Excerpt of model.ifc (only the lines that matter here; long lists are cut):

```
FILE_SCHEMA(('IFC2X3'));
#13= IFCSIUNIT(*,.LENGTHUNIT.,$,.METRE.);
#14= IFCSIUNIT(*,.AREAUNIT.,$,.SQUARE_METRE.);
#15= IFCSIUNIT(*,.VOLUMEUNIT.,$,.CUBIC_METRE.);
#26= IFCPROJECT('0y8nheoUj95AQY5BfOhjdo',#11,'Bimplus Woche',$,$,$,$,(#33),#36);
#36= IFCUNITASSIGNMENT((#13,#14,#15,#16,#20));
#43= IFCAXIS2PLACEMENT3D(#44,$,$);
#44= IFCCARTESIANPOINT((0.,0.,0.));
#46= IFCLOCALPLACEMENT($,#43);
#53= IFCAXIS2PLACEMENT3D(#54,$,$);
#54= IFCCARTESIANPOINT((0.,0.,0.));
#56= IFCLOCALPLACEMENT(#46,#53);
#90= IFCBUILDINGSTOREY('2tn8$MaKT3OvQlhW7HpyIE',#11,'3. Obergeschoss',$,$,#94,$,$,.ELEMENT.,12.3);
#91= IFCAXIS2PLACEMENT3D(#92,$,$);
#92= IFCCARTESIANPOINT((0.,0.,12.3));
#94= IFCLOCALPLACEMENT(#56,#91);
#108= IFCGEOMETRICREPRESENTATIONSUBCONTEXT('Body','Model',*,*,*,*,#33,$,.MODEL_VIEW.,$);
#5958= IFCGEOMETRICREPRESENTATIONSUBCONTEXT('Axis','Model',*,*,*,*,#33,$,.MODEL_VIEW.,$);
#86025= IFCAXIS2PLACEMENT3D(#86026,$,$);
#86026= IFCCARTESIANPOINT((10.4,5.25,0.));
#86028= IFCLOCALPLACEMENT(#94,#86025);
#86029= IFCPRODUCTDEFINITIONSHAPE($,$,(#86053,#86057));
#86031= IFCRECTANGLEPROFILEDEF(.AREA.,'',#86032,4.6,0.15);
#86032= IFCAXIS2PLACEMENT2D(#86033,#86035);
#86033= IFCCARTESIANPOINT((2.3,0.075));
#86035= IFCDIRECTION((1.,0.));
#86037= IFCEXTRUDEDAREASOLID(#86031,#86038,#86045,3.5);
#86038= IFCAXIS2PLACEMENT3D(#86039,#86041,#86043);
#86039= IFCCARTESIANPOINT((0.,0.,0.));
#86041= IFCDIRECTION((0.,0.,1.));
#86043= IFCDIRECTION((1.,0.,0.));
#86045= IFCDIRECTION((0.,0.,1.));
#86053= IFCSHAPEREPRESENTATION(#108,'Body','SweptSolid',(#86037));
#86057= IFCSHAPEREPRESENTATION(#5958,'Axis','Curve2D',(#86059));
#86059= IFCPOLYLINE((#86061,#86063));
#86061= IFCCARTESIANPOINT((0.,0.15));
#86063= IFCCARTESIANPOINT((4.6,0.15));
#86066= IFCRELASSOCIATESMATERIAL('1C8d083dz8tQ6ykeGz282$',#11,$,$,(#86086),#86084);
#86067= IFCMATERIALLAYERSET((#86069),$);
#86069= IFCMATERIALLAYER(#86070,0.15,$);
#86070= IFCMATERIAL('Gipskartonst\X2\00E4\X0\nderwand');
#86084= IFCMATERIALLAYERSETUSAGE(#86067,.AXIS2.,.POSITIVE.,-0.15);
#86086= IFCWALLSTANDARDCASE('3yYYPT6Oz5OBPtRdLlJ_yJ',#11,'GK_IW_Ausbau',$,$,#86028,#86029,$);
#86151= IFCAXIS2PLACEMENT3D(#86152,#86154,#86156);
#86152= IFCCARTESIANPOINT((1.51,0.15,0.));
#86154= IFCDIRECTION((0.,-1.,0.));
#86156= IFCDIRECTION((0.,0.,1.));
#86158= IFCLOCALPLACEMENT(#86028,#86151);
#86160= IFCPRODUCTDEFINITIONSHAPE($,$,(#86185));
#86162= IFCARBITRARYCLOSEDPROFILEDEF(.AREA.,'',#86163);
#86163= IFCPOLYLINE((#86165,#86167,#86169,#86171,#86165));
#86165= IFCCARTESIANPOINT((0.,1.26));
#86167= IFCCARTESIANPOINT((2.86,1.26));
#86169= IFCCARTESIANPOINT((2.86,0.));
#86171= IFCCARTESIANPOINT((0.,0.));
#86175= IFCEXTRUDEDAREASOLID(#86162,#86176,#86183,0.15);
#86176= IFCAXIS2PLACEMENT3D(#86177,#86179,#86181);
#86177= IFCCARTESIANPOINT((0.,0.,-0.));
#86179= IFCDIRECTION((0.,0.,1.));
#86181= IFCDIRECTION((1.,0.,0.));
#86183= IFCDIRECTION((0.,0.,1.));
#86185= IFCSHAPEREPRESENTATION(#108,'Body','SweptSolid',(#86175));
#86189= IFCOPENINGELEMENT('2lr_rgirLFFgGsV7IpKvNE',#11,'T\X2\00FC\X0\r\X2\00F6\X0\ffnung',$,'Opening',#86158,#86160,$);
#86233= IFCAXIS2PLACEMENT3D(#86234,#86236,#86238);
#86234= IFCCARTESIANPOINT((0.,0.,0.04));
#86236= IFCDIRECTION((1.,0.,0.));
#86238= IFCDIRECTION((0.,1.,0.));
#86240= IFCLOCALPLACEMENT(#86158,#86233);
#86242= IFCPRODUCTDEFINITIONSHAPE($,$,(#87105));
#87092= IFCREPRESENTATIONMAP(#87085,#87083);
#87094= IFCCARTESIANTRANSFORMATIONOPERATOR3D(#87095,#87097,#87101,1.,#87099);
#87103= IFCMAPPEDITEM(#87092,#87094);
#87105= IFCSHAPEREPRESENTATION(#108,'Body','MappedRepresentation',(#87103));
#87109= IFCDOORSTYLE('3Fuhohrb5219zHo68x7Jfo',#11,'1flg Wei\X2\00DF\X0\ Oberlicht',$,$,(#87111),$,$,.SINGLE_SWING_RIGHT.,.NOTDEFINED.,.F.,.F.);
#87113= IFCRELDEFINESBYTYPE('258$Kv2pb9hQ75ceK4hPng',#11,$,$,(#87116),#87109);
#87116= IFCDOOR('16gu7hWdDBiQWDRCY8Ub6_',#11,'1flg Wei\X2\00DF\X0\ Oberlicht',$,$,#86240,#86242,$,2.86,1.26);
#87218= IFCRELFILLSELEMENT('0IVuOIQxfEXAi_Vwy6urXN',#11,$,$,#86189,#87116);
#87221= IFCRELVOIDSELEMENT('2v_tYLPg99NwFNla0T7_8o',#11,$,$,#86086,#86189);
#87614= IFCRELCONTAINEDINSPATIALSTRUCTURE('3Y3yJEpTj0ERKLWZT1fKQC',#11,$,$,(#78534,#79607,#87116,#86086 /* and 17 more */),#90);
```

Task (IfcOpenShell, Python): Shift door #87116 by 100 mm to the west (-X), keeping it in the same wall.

```python
import ifcopenshell
import ifcopenshell.api.geometry
import ifcopenshell.util.placement
import ifcopenshell.util.unit

model = ifcopenshell.open("model.ifc")
unit_scale = ifcopenshell.util.unit.calculate_unit_scale(model)

door = model.by_guid("16gu7hWdDBiQWDRCY8Ub6_")
opening = door.FillsVoids[0].RelatingOpeningElement
wall = opening.VoidsElements[0].RelatingBuildingElement

wall_matrix = ifcopenshell.util.placement.get_local_placement(wall.ObjectPlacement)
shift = wall_matrix[:3, 0] * -0.1 / unit_scale
before = ifcopenshell.util.placement.get_local_placement(door.ObjectPlacement)[:3, 3].copy()

# The door is placed relative to its opening, so it follows when the opening moves.
matrix = ifcopenshell.util.placement.get_local_placement(opening.ObjectPlacement)
matrix[:3, 3] += shift
ifcopenshell.api.geometry.edit_object_placement(
    model, product=opening, matrix=matrix, is_si=False, should_transform_children=True
)

after = ifcopenshell.util.placement.get_local_placement(door.ObjectPlacement)[:3, 3]
print("door moved by", (after - before).round(3) + 0.0)

model.write("model-out.ifc")
```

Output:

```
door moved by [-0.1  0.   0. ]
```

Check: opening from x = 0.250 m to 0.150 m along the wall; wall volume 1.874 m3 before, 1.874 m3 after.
